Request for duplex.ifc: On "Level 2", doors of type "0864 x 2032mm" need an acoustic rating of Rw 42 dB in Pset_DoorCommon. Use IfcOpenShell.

First a look at what the model holds.

```python
import ifcopenshell
import ifcopenshell.util.element

model = ifcopenshell.open("duplex.ifc")
print(model.schema)
storey = next(s for s in model.by_type("IfcBuildingStorey") if s.Name == "Level 2")
doors = [e for e in ifcopenshell.util.element.get_decomposition(storey) if e.is_a("IfcDoor")]
seen = {}
for e in doors:
    element_type = ifcopenshell.util.element.get_type(e)
    key = (element_type.Name if element_type != e and element_type else None, ifcopenshell.util.element.get_pset(e, "Pset_DoorCommon", "AcousticRating"))
    seen[key] = seen.get(key, 0) + 1
for (name, value), count in sorted(seen.items(), key=str):
    print(count, "x", name, "|", value)
```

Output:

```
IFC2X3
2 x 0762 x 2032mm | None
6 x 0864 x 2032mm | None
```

```python
import ifcopenshell
import ifcopenshell.api.pset
import ifcopenshell.util.element

model = ifcopenshell.open("duplex.ifc")

storey = next(s for s in model.by_type("IfcBuildingStorey") if s.Name == "Level 2")
doors = [e for e in ifcopenshell.util.element.get_decomposition(storey) if e.is_a("IfcDoor")]

count = 0
for e in doors:
    element_type = ifcopenshell.util.element.get_type(e)
    if element_type in (None, e) or element_type.Name != "0864 x 2032mm":
        continue
    # add_pset returns the element's existing set when there is one.
    pset = ifcopenshell.api.pset.add_pset(model, product=e, name="Pset_DoorCommon")
    ifcopenshell.api.pset.edit_pset(model, pset=pset, properties={"AcousticRating": "Rw 42 dB"})
    count += 1

print(count, "doors updated")

model.write("duplex-out.ifc")
```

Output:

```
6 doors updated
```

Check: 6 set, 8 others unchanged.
